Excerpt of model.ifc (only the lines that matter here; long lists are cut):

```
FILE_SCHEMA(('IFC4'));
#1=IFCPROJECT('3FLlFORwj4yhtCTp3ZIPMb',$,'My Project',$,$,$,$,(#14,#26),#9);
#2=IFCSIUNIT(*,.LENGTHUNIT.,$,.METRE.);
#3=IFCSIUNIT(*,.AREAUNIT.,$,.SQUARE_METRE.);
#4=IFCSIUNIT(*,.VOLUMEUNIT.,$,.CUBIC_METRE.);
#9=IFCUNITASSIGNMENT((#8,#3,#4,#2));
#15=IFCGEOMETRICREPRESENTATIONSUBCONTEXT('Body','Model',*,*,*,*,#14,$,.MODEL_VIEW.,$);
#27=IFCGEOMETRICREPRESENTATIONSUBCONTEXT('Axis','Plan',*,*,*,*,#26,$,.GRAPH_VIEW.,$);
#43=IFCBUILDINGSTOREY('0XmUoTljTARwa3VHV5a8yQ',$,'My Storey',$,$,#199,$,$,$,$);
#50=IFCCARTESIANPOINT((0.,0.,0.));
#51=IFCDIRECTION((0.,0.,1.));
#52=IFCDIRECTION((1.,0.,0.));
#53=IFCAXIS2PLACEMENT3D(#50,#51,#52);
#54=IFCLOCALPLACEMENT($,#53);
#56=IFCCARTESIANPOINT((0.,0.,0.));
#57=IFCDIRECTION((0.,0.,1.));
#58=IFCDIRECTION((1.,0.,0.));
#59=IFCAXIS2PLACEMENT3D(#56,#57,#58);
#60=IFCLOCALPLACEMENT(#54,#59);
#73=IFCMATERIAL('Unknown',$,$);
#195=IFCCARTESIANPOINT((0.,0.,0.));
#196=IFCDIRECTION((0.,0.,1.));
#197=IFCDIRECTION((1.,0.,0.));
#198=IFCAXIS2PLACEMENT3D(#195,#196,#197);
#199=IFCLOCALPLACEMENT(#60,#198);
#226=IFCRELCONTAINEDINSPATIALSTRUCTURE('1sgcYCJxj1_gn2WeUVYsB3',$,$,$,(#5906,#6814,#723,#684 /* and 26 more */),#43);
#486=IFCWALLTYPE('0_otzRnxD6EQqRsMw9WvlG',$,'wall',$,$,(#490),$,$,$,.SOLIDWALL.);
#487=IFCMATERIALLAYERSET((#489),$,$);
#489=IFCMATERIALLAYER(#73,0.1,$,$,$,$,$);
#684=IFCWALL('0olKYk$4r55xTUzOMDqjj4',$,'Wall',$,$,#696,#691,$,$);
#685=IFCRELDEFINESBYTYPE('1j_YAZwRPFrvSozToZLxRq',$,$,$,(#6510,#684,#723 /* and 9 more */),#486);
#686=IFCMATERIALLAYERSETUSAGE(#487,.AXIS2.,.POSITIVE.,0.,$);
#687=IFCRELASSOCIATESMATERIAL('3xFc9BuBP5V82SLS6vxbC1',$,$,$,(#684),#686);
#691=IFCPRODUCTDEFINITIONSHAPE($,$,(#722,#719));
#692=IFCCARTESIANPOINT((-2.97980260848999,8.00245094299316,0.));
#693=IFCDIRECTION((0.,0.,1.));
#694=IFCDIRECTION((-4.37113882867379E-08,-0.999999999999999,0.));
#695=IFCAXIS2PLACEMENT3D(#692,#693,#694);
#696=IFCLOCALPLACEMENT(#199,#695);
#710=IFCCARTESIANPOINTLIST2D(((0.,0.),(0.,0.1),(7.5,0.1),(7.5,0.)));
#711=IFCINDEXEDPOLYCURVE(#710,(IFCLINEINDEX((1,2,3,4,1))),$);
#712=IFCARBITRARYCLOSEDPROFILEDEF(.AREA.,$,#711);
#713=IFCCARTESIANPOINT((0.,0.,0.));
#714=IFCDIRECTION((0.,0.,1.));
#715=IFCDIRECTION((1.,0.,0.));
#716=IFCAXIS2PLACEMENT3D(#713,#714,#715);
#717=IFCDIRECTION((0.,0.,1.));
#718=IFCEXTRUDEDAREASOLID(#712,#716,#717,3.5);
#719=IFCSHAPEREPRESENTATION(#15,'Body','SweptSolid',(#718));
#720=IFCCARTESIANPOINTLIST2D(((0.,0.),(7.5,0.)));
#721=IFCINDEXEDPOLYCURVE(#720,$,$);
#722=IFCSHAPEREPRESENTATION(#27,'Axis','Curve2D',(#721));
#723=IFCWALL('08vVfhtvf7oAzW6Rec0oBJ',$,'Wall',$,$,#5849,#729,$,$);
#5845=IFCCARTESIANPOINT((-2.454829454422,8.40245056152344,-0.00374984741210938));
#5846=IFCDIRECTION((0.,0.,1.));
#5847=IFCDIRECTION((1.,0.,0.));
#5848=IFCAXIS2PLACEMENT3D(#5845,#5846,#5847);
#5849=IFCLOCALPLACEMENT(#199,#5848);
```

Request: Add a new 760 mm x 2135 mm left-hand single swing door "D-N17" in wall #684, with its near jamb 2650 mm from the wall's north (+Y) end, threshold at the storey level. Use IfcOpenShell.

```python
import numpy as np
import ifcopenshell
import ifcopenshell.api.feature
import ifcopenshell.api.geometry
import ifcopenshell.api.root
import ifcopenshell.api.spatial
import ifcopenshell.geom
import ifcopenshell.util.element
import ifcopenshell.util.placement
import ifcopenshell.util.representation
import ifcopenshell.util.shape
import ifcopenshell.util.unit

model = ifcopenshell.open("model.ifc")
unit_scale = ifcopenshell.util.unit.calculate_unit_scale(model)
settings = ifcopenshell.geom.settings()


def volume(element):
    """Net volume in cubic metres, openings subtracted."""
    shape = ifcopenshell.geom.create_shape(settings, element)
    return ifcopenshell.util.shape.get_volume(shape.geometry)


wall = model.by_id(684)
storey = ifcopenshell.util.element.get_container(wall, ifc_class="IfcBuildingStorey")
context = ifcopenshell.util.representation.get_context(model, "Model", "Body", "MODEL_VIEW")
before = volume(wall)

width, height, from_end, sill = 0.76, 2.135, 2.65, 0.0  # metres

# The wall runs along its own X axis, and the end named is its -X end.
wall_shape = ifcopenshell.geom.create_shape(settings, wall)
x, y, z = ifcopenshell.util.shape.get_vertices(wall_shape.geometry).T
start = x.min() + from_end
face, thickness = float(y.min()), float(y.max() - y.min())
wall_matrix = ifcopenshell.util.placement.get_local_placement(wall.ObjectPlacement)
level = ifcopenshell.util.placement.get_local_placement(storey.ObjectPlacement)[2, 3]


def in_wall(x, y):
    """Placement at x, y metres in the wall's axes, at sill height."""
    matrix = wall_matrix.copy()
    matrix[:, 3] = wall_matrix @ np.array([x / unit_scale, y / unit_scale, 0.0, 1.0])
    matrix[2, 3] = level + sill / unit_scale
    return matrix


# Opening: a box that overshoots both wall faces by 50 mm.
opening = ifcopenshell.api.root.create_entity(model, ifc_class="IfcOpeningElement", predefined_type="OPENING")
box = ifcopenshell.api.geometry.add_wall_representation(
    model, context=context, length=width, height=height, thickness=thickness + 0.1
)
ifcopenshell.api.geometry.assign_representation(model, product=opening, representation=box)
ifcopenshell.api.geometry.edit_object_placement(model, product=opening, matrix=in_wall(start, face - 0.05), is_si=False)
ifcopenshell.api.feature.add_feature(model, feature=opening, element=wall)

door = ifcopenshell.api.root.create_entity(model, ifc_class="IfcDoor", name="D-N17", predefined_type="DOOR")
door.OverallWidth, door.OverallHeight = width / unit_scale, height / unit_scale
door.OperationType = "SINGLE_SWING_LEFT"
body = ifcopenshell.api.geometry.add_door_representation(
    model,
    context=context,
    overall_width=door.OverallWidth,
    overall_height=door.OverallHeight,
    operation_type="SINGLE_SWING_LEFT",
    lining_properties={"LiningDepth": thickness / unit_scale, "ThresholdDepth": thickness / unit_scale},
)
ifcopenshell.api.geometry.assign_representation(model, product=door, representation=body)
ifcopenshell.api.spatial.assign_container(model, products=[door], relating_structure=storey)
ifcopenshell.api.feature.add_filling(model, opening=opening, element=door)

# The lining spans the wall, so the door starts at the wall face.
ifcopenshell.api.geometry.edit_object_placement(model, product=door, matrix=in_wall(start, face), is_si=False)

after = volume(wall)

print(f"wall volume {before:.3f} -> {after:.3f} m3")

model.write("model_updated.ifc")
```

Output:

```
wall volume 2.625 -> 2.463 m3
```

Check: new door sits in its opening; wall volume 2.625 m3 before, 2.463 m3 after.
